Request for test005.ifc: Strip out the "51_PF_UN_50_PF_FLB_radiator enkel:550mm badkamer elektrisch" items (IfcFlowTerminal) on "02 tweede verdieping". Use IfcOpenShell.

First a look at what the model holds.

```python
import ifcopenshell
import ifcopenshell.util.element

model = ifcopenshell.open("test005.ifc")
print(model.schema)
storey = next(s for s in model.by_type("IfcBuildingStorey") if s.Name == "02 tweede verdieping")
terminals = [e for e in ifcopenshell.util.element.get_decomposition(storey) if e.is_a("IfcFlowTerminal")]
seen = {}
for e in terminals:
    element_type = ifcopenshell.util.element.get_type(e)
    name = element_type.Name if element_type not in (None, e) else None
    seen[name] = seen.get(name, 0) + 1
for name, count in sorted(seen.items(), key=str):
    print(count, "x", name)
```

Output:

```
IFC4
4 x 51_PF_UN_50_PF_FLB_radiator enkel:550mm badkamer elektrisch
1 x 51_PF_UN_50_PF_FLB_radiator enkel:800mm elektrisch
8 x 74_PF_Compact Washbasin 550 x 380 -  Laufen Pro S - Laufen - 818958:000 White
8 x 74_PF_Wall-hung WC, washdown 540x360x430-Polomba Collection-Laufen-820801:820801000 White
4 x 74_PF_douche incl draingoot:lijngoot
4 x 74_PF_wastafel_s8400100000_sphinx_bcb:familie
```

```python
import ifcopenshell
import ifcopenshell.api.root
import ifcopenshell.util.element

model = ifcopenshell.open("test005.ifc")

storey = next(s for s in model.by_type("IfcBuildingStorey") if s.Name == "02 tweede verdieping")
terminals = [e for e in ifcopenshell.util.element.get_decomposition(storey) if e.is_a("IfcFlowTerminal")]
targets = [e for e in terminals if (t := ifcopenshell.util.element.get_type(e)) not in (None, e) and t.Name == "51_PF_UN_50_PF_FLB_radiator enkel:550mm badkamer elektrisch"]

for e in targets:
    ifcopenshell.api.root.remove_product(model, product=e)
print(len(targets), "removed")

model.write("test005_edited.ifc")
```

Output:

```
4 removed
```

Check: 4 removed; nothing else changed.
